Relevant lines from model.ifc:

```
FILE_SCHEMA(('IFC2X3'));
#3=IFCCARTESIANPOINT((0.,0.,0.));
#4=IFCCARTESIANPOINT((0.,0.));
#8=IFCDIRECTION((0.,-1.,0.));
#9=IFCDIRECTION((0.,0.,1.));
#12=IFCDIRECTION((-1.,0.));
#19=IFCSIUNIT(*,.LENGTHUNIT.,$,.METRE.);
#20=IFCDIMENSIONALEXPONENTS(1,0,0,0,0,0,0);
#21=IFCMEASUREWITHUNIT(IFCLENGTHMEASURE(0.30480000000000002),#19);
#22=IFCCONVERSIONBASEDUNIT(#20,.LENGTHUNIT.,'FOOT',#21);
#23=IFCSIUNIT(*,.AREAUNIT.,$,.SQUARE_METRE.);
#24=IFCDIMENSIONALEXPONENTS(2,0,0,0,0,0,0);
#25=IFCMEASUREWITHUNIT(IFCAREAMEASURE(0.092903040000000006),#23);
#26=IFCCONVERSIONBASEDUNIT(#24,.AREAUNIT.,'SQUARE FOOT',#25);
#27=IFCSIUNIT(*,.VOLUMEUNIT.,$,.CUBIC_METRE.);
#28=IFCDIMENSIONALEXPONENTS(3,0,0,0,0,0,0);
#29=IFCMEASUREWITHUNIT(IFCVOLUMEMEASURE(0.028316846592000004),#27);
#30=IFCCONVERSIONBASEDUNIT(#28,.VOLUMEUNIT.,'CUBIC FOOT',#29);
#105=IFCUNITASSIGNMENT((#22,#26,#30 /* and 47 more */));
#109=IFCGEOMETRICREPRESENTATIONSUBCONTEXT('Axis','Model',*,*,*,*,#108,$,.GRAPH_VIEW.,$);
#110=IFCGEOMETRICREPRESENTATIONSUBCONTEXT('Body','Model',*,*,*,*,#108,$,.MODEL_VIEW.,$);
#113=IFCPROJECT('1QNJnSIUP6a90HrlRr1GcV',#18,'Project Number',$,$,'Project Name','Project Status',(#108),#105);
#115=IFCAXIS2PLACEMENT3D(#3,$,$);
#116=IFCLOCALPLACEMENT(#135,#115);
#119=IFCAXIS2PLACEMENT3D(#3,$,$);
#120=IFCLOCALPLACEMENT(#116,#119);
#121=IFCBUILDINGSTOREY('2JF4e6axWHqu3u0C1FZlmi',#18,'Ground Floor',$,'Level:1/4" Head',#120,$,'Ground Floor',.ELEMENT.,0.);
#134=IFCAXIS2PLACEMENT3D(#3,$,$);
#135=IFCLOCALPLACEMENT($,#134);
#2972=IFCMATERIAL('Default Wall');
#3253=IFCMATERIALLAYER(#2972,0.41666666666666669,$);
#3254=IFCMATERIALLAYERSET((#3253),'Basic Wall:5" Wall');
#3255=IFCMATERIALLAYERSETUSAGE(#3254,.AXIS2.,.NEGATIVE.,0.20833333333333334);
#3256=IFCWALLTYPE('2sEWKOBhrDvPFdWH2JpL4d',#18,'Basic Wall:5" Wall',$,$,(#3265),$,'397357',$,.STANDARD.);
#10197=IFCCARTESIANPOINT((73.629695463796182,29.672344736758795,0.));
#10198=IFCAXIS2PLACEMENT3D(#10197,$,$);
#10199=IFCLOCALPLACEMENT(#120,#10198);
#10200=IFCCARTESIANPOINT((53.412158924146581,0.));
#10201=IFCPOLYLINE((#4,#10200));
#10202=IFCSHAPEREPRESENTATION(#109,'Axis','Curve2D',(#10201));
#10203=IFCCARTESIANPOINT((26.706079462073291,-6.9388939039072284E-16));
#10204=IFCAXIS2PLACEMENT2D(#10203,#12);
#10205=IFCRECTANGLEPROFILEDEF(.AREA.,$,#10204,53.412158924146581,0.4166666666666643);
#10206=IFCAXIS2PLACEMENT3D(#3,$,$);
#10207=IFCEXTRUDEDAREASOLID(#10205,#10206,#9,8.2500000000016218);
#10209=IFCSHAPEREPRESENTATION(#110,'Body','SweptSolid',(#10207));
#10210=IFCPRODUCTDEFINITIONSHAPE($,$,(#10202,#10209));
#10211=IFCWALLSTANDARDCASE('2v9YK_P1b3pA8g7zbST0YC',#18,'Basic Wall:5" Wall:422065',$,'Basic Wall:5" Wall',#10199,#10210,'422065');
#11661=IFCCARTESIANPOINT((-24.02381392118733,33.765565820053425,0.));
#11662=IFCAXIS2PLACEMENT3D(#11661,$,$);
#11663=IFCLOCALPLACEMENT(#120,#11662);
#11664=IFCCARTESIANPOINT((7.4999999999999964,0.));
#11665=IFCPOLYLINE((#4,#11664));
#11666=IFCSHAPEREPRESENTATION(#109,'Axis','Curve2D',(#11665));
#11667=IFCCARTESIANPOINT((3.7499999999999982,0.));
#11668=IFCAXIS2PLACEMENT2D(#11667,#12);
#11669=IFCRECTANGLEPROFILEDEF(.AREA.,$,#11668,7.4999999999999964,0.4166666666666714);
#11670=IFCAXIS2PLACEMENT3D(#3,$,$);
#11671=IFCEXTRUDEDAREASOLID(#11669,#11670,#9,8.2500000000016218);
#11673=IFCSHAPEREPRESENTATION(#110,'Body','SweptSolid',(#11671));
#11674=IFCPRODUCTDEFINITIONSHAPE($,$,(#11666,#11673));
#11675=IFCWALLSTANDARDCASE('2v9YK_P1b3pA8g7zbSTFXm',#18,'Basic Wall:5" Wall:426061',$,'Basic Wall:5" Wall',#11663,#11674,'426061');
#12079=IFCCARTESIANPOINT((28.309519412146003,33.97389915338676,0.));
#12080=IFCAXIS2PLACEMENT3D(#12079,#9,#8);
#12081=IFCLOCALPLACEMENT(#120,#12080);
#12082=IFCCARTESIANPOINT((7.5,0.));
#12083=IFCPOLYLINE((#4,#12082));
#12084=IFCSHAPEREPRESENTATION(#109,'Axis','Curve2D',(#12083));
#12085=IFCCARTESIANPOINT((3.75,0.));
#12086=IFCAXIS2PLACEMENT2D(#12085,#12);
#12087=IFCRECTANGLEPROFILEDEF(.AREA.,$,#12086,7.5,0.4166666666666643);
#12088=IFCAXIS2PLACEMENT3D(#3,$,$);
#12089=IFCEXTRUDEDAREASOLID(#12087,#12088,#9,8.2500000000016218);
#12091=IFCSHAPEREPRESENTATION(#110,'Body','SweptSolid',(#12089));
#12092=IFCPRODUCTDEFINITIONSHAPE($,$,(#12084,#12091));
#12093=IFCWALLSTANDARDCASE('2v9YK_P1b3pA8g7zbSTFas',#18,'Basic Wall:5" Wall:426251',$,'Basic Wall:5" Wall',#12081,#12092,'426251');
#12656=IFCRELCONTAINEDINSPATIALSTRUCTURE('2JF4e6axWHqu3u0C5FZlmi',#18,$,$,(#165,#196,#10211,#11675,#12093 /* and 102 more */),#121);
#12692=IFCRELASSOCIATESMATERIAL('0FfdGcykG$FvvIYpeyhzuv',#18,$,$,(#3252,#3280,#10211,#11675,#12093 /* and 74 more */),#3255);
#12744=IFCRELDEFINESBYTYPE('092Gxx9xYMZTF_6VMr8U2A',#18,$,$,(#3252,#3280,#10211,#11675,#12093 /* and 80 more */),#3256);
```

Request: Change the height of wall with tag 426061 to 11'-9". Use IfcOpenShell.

```python
import ifcopenshell
import ifcopenshell.geom
import ifcopenshell.util.representation
import ifcopenshell.util.shape
import ifcopenshell.util.unit

model = ifcopenshell.open("model.ifc")
unit_scale = ifcopenshell.util.unit.calculate_unit_scale(model)
settings = ifcopenshell.geom.settings()


def volume(element):
    """Net volume in cubic metres, openings subtracted."""
    shape = ifcopenshell.geom.create_shape(settings, element)
    return ifcopenshell.util.shape.get_volume(shape.geometry)


wall = model.by_id(11675)
before = volume(wall)

body = ifcopenshell.util.representation.get_representation(wall, "Model", "Body")
solid = body.Items[0]
old_height = solid.Depth
solid.Depth = 141 * 0.0254 / unit_scale
after = volume(wall)

print(f"height {old_height:g} -> {solid.Depth:g}, volume {before:.3f} -> {after:.3f} m3")

model.write("model_updated.ifc")
```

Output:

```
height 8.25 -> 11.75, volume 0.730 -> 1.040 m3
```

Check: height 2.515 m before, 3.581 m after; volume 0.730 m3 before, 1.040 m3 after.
